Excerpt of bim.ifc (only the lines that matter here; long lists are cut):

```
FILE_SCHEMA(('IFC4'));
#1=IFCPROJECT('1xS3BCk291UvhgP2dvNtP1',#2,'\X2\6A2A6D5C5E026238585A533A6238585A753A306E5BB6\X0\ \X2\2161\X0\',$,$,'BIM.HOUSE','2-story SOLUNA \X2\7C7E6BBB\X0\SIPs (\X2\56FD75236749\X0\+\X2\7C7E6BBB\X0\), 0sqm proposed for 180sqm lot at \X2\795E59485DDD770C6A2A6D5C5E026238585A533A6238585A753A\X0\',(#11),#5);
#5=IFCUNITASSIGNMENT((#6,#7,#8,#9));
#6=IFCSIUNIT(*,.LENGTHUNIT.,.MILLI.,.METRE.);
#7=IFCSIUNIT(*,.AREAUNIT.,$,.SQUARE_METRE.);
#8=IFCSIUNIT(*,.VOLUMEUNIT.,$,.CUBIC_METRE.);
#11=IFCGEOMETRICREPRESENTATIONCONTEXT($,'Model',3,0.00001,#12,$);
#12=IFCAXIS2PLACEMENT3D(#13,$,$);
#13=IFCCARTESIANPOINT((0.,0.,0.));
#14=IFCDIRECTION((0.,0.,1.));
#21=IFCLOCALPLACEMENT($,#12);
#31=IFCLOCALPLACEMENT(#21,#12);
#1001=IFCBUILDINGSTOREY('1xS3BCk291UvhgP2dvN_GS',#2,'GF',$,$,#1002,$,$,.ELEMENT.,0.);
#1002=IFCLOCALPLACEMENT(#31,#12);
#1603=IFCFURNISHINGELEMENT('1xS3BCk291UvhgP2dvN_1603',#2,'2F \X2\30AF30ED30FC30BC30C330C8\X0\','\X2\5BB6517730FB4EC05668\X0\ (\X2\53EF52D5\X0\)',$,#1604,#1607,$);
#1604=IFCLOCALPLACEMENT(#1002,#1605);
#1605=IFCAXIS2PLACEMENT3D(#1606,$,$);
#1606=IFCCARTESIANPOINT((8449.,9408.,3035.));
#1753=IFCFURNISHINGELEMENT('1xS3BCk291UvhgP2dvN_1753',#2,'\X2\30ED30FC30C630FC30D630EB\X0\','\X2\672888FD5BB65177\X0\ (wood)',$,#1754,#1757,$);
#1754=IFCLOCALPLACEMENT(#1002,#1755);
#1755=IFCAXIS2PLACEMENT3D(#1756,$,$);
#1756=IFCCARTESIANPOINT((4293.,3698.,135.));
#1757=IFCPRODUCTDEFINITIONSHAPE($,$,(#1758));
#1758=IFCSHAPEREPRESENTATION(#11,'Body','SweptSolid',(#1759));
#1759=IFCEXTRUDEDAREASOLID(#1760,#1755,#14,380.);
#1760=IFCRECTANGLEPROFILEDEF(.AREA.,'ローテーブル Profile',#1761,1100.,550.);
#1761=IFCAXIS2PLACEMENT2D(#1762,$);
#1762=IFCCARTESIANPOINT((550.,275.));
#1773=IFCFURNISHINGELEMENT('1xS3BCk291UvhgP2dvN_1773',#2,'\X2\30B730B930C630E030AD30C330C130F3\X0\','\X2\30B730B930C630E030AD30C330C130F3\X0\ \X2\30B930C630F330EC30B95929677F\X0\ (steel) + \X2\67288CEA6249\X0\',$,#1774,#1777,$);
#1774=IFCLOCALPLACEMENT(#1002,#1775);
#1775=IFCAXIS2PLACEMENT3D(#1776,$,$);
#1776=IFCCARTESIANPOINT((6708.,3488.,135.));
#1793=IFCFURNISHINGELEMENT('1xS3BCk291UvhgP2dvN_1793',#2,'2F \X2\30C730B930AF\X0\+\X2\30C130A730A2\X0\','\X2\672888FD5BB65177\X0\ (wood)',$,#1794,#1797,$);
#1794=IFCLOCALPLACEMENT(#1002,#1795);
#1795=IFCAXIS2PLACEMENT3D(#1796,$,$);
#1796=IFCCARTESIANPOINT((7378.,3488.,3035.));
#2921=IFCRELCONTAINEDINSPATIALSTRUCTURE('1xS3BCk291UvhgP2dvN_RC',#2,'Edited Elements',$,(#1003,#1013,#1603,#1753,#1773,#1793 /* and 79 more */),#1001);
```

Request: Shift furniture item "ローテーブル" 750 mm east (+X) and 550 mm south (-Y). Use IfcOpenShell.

```python
import ifcopenshell
import ifcopenshell.api.geometry
import ifcopenshell.util.placement

model = ifcopenshell.open("bim.ifc")

item = model.by_id(1753)
matrix = ifcopenshell.util.placement.get_local_placement(item.ObjectPlacement)
matrix[0, 3] += 750.0
matrix[1, 3] -= 550.0
ifcopenshell.api.geometry.edit_object_placement(model, product=item, matrix=matrix, is_si=False)

print(ifcopenshell.util.placement.get_local_placement(item.ObjectPlacement).round(3) + 0.0)

model.write("bim_v2.ifc")
```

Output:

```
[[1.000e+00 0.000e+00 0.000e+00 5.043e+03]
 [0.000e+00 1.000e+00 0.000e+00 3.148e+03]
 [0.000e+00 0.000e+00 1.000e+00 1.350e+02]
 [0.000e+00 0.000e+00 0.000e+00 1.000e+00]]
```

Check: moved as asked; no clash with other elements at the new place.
